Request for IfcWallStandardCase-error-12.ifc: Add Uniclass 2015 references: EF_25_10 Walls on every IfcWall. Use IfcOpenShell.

First a look at what the model holds.

```python
import ifcopenshell

model = ifcopenshell.open("IfcWallStandardCase-error-12.ifc")
print(model.schema)
print("classifications:", [c.Name for c in model.by_type("IfcClassification")])
for ifc_class in ("IfcDoor", "IfcRoof", "IfcStair", "IfcWall", "IfcWindow"):
    print(ifc_class, len(model.by_type(ifc_class)))
```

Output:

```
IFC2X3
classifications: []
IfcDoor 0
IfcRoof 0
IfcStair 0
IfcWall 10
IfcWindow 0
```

```python
import ifcopenshell
import ifcopenshell.api.classification

model = ifcopenshell.open("IfcWallStandardCase-error-12.ifc")

# IFC2X3 requires Source and Edition and has no link from the project to the system.
system = model.create_entity("IfcClassification", Source="NBS", Edition="2015", Name="Uniclass 2015")

codes = {
    "IfcWall": ("EF_25_10", "Walls"),
}
for ifc_class, (code, name) in codes.items():
    products = model.by_type(ifc_class)
    ifcopenshell.api.classification.add_reference(
        model, products=products, classification=system, identification=code, name=name
    )
    print(code, len(products))

model.write("IfcWallStandardCase-error-12_updated.ifc")
```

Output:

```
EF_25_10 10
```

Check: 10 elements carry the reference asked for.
